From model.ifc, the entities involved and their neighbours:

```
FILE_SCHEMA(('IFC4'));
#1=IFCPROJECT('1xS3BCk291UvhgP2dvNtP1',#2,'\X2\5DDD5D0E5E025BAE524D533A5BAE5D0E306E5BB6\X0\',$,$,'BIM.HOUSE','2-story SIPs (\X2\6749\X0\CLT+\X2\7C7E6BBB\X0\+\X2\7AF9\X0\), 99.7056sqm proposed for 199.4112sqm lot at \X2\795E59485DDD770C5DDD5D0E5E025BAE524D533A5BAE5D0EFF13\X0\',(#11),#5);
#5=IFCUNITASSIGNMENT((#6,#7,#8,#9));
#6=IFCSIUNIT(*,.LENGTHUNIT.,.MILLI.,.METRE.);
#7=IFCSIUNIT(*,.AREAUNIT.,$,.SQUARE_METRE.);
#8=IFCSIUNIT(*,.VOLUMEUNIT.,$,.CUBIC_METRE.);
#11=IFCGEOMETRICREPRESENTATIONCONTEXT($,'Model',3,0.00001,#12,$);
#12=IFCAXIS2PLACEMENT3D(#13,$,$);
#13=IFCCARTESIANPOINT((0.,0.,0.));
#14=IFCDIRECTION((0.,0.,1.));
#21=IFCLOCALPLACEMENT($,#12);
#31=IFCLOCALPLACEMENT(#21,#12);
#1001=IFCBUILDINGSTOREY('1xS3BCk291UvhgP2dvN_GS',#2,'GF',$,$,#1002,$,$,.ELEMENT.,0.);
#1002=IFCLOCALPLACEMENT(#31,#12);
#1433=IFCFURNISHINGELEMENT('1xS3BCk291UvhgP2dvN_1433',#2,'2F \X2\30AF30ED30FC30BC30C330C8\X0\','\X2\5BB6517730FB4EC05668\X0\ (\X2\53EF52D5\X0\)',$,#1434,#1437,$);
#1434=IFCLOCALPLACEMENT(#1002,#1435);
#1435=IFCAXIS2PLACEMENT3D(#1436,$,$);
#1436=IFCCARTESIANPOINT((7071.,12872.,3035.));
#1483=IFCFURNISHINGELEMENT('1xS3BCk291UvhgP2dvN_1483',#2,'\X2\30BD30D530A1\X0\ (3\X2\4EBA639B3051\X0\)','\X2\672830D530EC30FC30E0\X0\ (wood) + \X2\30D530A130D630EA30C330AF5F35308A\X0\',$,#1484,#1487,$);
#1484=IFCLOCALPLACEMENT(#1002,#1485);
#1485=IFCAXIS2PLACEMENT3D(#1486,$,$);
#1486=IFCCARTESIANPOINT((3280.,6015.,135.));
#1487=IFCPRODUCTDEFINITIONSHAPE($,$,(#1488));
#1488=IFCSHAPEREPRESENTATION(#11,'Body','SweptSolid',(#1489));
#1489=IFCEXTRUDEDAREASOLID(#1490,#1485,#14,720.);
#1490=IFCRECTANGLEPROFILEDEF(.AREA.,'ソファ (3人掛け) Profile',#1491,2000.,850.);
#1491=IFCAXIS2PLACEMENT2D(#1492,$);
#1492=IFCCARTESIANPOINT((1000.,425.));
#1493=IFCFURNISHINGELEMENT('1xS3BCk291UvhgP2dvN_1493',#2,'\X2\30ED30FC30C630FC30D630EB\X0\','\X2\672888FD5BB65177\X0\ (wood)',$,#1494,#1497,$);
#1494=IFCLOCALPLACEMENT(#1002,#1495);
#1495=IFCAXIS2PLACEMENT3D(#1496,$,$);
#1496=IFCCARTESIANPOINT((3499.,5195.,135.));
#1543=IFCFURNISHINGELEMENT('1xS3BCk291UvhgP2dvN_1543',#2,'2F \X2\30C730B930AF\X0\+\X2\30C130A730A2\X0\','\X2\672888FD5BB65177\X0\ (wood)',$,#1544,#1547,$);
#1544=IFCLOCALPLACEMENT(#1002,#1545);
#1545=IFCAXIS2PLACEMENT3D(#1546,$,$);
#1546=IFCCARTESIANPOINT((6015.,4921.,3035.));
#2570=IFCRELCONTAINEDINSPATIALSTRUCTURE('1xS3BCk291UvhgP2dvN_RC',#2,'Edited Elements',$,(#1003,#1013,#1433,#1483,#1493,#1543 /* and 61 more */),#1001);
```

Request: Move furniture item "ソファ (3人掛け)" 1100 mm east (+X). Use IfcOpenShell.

```python
import ifcopenshell
import ifcopenshell.api.geometry
import ifcopenshell.util.placement
import ifcopenshell.util.unit

model = ifcopenshell.open("model.ifc")
unit_scale = ifcopenshell.util.unit.calculate_unit_scale(model)

item = model.by_guid("1xS3BCk291UvhgP2dvN_1483")
matrix = ifcopenshell.util.placement.get_local_placement(item.ObjectPlacement)
matrix[0, 3] += 1.1 / unit_scale
ifcopenshell.api.geometry.edit_object_placement(model, product=item, matrix=matrix, is_si=False)

print(ifcopenshell.util.placement.get_local_placement(item.ObjectPlacement).round(3) + 0.0)

model.write("model_updated.ifc")
```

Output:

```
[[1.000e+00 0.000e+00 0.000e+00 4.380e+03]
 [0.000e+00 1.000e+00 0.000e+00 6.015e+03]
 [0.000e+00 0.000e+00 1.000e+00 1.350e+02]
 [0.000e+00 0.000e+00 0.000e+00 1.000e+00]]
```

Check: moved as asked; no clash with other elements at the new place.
